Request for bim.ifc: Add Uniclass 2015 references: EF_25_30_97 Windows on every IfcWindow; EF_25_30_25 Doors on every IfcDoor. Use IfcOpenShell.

First a look at what the model holds.

```python
import ifcopenshell

model = ifcopenshell.open("bim.ifc")
print(model.schema)
print("classifications:", [c.Name for c in model.by_type("IfcClassification")])
for ifc_class in ("IfcDoor", "IfcRoof", "IfcStair", "IfcWall", "IfcWindow"):
    print(ifc_class, len(model.by_type(ifc_class)))
```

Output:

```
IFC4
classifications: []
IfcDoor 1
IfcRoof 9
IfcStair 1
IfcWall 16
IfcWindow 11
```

```python
import ifcopenshell
import ifcopenshell.api.classification

model = ifcopenshell.open("bim.ifc")

system = ifcopenshell.api.classification.add_classification(model, classification="Uniclass 2015")

codes = {
    "IfcWindow": ("EF_25_30_97", "Windows"),
    "IfcDoor": ("EF_25_30_25", "Doors"),
}
for ifc_class, (code, name) in codes.items():
    products = model.by_type(ifc_class)
    ifcopenshell.api.classification.add_reference(
        model, products=products, classification=system, identification=code, name=name
    )
    print(code, len(products))

model.write("bim_rev.ifc")
```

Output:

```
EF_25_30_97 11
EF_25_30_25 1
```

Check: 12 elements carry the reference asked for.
